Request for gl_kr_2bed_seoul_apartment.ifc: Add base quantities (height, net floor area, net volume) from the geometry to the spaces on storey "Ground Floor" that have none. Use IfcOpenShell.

First a look at what the model holds.

```python
import ifcopenshell
import ifcopenshell.util.element
import ifcopenshell.util.unit

model = ifcopenshell.open("gl_kr_2bed_seoul_apartment.ifc")
print(model.schema)
for unit_type in ("LENGTHUNIT", "AREAUNIT", "VOLUMEUNIT"):
    print(unit_type, ifcopenshell.util.unit.calculate_unit_scale(model, unit_type))
storey = next(s for s in model.by_type("IfcBuildingStorey") if s.Name == "Ground Floor")
spaces = [e for e in ifcopenshell.util.element.get_decomposition(storey) if e.is_a("IfcSpace")]
for e in sorted(spaces, key=lambda e: e.id()):
    print(e.id(), e.is_a(), e.Name, list(ifcopenshell.util.element.get_psets(e, qtos_only=True)), sep=" | ")
```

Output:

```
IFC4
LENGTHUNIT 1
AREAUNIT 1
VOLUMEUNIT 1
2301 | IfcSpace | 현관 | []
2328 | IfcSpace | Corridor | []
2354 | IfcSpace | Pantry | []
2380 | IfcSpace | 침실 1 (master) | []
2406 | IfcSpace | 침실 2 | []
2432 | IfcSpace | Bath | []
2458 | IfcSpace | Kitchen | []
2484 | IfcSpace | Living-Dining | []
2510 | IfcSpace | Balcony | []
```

```python
import ifcopenshell
import ifcopenshell.api.pset
import ifcopenshell.geom
import ifcopenshell.util.element
import ifcopenshell.util.shape
import ifcopenshell.util.unit

model = ifcopenshell.open("gl_kr_2bed_seoul_apartment.ifc")
unit_scale = ifcopenshell.util.unit.calculate_unit_scale(model)
area_scale = ifcopenshell.util.unit.calculate_unit_scale(model, "AREAUNIT")
volume_scale = ifcopenshell.util.unit.calculate_unit_scale(model, "VOLUMEUNIT")
settings = ifcopenshell.geom.settings()

storey = next(s for s in model.by_type("IfcBuildingStorey") if s.Name == "Ground Floor")
spaces = [e for e in ifcopenshell.util.element.get_decomposition(storey) if e.is_a("IfcSpace")]

for e in sorted(spaces, key=lambda e: e.id()):
    if ifcopenshell.util.element.get_psets(e, qtos_only=True, should_inherit=False):
        continue
    # Geometry comes back in metres, in the element's own axes.
    shape = ifcopenshell.geom.create_shape(settings, e)
    values = {
        "Height": ifcopenshell.util.shape.get_z(shape.geometry) / unit_scale,
        "NetFloorArea": ifcopenshell.util.shape.get_footprint_area(shape.geometry) / area_scale,
        "NetVolume": ifcopenshell.util.shape.get_volume(shape.geometry) / volume_scale,
    }
    qto = ifcopenshell.api.pset.add_qto(model, product=e, name="Qto_SpaceBaseQuantities")
    ifcopenshell.api.pset.edit_qto(model, qto=qto, properties=values)
    print(e.id(), {k: round(v, 3) for k, v in values.items()})

model.write("gl_kr_2bed_seoul_apartment_edited.ifc")
```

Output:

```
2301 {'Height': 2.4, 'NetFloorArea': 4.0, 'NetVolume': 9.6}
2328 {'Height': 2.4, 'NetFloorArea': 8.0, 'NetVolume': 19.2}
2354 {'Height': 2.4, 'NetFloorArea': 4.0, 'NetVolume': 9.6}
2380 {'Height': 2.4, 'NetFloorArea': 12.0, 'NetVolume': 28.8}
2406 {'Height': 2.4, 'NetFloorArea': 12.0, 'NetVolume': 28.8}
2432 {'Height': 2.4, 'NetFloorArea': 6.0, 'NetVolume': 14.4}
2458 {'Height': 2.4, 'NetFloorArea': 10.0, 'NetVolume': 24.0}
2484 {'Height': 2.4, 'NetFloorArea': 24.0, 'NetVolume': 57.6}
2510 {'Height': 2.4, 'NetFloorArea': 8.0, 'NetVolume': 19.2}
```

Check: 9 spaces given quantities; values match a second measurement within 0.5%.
